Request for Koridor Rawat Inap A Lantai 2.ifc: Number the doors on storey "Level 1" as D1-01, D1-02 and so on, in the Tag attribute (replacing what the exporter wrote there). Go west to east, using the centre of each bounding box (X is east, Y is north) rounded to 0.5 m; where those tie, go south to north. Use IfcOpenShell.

First a look at what the model holds.

```python
import ifcopenshell
import ifcopenshell.util.element
import ifcopenshell.util.placement

model = ifcopenshell.open("Koridor Rawat Inap A Lantai 2.ifc")
print(model.schema)
storey = next(s for s in model.by_type("IfcBuildingStorey") if s.Name == "Level 1")
doors = [e for e in ifcopenshell.util.element.get_decomposition(storey) if e.is_a("IfcDoor")]
for e in sorted(doors, key=lambda e: e.id()):
    origin = ifcopenshell.util.placement.get_local_placement(e.ObjectPlacement)[:3, 3]
    print(e.id(), e.Tag, e.Name, origin.round(2) + 0.0, sep=" | ")
```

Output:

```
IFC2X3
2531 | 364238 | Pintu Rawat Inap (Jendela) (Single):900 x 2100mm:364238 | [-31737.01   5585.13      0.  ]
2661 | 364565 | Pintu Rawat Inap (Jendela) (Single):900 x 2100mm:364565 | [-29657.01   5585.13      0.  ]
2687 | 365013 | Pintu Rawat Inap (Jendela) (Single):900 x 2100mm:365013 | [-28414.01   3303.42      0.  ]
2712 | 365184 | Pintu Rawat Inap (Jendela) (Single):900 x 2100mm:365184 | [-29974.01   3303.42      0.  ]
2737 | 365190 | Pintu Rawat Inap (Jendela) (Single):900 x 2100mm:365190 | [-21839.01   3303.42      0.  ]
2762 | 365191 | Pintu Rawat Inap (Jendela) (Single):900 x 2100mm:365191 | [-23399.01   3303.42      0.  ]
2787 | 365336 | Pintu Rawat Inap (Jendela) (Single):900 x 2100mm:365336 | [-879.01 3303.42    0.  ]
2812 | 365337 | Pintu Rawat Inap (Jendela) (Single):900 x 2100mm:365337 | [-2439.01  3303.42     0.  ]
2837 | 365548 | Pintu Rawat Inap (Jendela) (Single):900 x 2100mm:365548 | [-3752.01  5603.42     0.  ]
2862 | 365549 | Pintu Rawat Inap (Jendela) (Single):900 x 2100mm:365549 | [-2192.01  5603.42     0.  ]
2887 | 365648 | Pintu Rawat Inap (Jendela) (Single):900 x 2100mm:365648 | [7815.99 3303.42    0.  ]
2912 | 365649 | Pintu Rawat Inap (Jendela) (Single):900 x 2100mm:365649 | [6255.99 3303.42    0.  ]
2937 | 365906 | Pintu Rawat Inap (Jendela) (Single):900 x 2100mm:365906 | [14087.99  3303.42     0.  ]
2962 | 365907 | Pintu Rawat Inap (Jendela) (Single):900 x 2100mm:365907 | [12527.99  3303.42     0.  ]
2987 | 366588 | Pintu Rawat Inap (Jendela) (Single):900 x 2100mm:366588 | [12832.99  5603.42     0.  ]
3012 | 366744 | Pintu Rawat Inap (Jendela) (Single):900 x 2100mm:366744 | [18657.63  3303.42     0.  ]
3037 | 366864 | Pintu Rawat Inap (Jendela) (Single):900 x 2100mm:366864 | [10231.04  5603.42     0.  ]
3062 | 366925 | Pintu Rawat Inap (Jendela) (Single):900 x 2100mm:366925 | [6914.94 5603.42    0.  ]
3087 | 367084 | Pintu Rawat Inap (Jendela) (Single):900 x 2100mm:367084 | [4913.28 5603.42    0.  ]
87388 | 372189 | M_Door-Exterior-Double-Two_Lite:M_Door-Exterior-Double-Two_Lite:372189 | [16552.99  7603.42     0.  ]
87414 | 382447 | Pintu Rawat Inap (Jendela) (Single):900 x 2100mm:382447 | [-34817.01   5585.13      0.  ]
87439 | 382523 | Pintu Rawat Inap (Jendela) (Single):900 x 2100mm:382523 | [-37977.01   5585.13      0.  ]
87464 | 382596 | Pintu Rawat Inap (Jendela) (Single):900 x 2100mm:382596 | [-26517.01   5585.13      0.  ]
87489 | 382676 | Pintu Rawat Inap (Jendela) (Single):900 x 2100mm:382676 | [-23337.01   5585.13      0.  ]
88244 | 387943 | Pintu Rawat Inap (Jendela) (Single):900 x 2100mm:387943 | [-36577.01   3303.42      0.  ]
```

```python
import ifcopenshell
import ifcopenshell.geom
import ifcopenshell.util.element
import ifcopenshell.util.shape

model = ifcopenshell.open("Koridor Rawat Inap A Lantai 2.ifc")
settings = ifcopenshell.geom.settings()
settings.set("use-world-coords", True)


def centre(element):
    shape = ifcopenshell.geom.create_shape(settings, element)
    return ifcopenshell.util.shape.get_bbox_centroid(shape.geometry)


storey = next(s for s in model.by_type("IfcBuildingStorey") if s.Name == "Level 1")
doors = [e for e in ifcopenshell.util.element.get_decomposition(storey) if e.is_a("IfcDoor")]

# Insertion points can sit at a corner or the storey origin, so sort by the geometry (in metres).
centres = {e: centre(e) for e in doors}
doors.sort(key=lambda e: (round(centres[e][0] / 0.5), centres[e][1]))

for i, e in enumerate(doors, start=1):
    number = f"D1-{i:02d}"
    e.Tag = number
    print(e.id(), number)

model.write("Koridor Rawat Inap A Lantai 2_rev.ifc")
```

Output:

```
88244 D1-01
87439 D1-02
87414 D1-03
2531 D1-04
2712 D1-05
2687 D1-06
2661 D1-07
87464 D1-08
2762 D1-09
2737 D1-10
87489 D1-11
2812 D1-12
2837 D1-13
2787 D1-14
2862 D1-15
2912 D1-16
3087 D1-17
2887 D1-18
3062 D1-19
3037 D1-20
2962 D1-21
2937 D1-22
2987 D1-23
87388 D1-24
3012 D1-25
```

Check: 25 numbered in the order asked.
